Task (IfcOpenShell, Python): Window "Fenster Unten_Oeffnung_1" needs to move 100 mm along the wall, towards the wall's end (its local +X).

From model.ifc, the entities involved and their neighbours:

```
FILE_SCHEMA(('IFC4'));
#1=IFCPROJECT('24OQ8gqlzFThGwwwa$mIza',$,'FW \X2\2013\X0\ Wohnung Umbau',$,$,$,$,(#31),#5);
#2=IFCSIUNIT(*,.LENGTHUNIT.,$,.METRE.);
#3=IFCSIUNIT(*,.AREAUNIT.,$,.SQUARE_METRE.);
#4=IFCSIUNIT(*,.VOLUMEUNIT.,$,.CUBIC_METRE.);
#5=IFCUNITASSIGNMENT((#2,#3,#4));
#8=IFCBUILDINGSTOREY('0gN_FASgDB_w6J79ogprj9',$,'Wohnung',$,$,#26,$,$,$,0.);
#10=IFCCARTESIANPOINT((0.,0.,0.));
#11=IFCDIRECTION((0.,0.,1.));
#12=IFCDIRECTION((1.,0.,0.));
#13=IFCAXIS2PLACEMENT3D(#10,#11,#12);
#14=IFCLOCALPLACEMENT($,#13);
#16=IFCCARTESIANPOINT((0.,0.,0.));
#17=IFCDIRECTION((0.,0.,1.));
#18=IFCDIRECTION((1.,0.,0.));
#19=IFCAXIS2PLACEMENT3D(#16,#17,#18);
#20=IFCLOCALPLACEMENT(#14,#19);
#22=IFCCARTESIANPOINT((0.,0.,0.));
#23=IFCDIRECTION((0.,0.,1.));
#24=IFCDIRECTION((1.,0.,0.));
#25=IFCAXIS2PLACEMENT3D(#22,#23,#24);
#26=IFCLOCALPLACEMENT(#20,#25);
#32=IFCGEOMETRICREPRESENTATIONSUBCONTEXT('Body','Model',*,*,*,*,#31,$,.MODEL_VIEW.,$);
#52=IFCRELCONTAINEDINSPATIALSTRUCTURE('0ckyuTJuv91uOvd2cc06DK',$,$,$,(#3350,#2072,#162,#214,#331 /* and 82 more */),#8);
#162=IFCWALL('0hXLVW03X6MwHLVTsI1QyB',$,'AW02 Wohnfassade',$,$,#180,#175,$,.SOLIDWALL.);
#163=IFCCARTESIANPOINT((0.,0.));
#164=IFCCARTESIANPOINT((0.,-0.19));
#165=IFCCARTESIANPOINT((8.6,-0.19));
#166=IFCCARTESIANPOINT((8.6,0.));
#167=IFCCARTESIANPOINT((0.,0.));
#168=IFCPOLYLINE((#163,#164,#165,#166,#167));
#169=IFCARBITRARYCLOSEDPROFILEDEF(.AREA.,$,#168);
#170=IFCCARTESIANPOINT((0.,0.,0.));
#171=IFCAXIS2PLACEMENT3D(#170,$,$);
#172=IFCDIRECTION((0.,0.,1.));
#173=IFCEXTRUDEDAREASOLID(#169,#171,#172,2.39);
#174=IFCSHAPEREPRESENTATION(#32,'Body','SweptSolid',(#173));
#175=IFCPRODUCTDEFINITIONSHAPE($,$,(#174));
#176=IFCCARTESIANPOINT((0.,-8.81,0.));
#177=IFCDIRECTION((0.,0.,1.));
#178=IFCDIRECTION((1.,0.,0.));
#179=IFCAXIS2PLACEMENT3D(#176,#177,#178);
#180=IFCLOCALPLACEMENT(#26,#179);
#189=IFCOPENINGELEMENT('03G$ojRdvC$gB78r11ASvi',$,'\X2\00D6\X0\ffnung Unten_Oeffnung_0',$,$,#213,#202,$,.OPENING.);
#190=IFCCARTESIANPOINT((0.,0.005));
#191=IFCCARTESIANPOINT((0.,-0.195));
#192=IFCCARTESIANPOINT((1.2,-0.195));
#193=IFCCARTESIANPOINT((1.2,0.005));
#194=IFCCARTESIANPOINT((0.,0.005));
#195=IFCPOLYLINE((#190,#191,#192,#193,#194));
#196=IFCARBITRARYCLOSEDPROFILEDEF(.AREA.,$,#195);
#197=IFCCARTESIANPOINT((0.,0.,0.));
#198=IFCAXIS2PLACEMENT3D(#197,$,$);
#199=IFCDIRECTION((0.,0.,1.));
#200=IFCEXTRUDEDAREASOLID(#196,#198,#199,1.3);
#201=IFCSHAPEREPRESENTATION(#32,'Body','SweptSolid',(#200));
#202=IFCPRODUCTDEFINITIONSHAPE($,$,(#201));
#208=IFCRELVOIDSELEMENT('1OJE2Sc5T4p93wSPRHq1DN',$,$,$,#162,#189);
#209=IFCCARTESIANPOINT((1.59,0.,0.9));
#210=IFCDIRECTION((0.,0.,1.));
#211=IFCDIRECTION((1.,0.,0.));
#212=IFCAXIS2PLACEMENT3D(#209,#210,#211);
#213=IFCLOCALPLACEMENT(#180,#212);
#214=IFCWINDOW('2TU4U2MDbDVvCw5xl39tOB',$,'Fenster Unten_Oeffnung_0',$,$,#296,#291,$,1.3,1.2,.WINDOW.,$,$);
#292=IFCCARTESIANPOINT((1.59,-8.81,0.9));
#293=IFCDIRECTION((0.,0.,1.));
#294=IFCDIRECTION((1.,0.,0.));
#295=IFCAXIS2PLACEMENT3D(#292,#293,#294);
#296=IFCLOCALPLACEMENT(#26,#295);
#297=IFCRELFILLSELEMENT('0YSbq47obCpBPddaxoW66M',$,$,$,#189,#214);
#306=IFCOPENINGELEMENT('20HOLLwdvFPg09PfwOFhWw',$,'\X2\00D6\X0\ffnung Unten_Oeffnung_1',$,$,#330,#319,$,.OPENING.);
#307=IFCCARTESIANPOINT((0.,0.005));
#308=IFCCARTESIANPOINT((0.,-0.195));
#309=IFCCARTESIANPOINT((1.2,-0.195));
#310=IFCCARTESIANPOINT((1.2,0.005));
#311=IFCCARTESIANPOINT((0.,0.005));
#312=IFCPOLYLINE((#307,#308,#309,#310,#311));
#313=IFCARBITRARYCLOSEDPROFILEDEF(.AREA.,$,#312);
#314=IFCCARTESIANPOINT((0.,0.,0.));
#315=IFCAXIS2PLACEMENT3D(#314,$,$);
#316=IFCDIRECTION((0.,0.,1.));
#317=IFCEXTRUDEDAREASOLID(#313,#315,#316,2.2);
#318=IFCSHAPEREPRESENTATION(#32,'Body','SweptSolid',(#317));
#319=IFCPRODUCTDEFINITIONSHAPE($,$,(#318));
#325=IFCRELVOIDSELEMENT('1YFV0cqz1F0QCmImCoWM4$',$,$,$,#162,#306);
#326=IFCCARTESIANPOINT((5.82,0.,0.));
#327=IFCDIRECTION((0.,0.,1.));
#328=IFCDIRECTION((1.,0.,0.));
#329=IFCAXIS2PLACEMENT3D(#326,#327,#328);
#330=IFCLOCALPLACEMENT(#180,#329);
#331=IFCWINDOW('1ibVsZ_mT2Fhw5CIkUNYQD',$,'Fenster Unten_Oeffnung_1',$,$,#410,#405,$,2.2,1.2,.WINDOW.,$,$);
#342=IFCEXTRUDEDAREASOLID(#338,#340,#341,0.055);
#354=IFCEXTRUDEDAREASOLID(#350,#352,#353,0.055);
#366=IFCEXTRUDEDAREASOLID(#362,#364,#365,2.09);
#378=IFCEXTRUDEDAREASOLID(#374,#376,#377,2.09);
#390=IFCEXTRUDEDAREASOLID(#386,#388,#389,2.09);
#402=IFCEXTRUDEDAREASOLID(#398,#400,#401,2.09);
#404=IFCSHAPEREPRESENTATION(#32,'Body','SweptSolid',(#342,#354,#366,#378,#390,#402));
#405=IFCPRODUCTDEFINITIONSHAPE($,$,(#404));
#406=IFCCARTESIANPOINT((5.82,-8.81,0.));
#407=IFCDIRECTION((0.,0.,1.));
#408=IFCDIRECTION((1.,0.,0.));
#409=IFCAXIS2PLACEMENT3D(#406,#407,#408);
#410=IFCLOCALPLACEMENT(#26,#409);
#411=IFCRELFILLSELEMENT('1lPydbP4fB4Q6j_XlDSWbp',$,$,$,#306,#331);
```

```python
import ifcopenshell
import ifcopenshell.api.geometry
import ifcopenshell.util.placement
import ifcopenshell.util.unit

model = ifcopenshell.open("model.ifc")
unit_scale = ifcopenshell.util.unit.calculate_unit_scale(model)

window = model.by_guid("1ibVsZ_mT2Fhw5CIkUNYQD")
opening = window.FillsVoids[0].RelatingOpeningElement
wall = opening.VoidsElements[0].RelatingBuildingElement

wall_matrix = ifcopenshell.util.placement.get_local_placement(wall.ObjectPlacement)
shift = wall_matrix[:3, 0] * 0.1 / unit_scale
before = ifcopenshell.util.placement.get_local_placement(window.ObjectPlacement)[:3, 3].copy()

# The window is not placed relative to its opening, so move both.
for product in (opening, window):
    matrix = ifcopenshell.util.placement.get_local_placement(product.ObjectPlacement)
    matrix[:3, 3] += shift
    ifcopenshell.api.geometry.edit_object_placement(model, product=product, matrix=matrix, is_si=False)

after = ifcopenshell.util.placement.get_local_placement(window.ObjectPlacement)[:3, 3]
print("window moved by", (after - before).round(3) + 0.0)

model.write("model_v2.ifc")
```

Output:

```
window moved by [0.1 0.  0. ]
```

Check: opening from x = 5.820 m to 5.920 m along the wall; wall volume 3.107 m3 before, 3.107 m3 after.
